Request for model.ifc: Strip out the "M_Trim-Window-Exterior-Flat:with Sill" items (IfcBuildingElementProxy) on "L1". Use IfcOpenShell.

First a look at what the model holds.

```python
import ifcopenshell
import ifcopenshell.util.element

model = ifcopenshell.open("model.ifc")
print(model.schema)
storey = next(s for s in model.by_type("IfcBuildingStorey") if s.Name == "L1")
proxies = [e for e in ifcopenshell.util.element.get_decomposition(storey) if e.is_a("IfcBuildingElementProxy")]
seen = {}
for e in proxies:
    element_type = ifcopenshell.util.element.get_type(e)
    name = element_type.Name if element_type not in (None, e) else None
    seen[name] = seen.get(name, 0) + 1
for name, count in sorted(seen.items(), key=str):
    print(count, "x", name)
```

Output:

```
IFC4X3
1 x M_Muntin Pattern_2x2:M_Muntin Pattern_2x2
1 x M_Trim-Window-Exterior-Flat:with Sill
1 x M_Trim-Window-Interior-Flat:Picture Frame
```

```python
import ifcopenshell
import ifcopenshell.api.root
import ifcopenshell.util.element

model = ifcopenshell.open("model.ifc")

storey = next(s for s in model.by_type("IfcBuildingStorey") if s.Name == "L1")
proxies = [e for e in ifcopenshell.util.element.get_decomposition(storey) if e.is_a("IfcBuildingElementProxy")]
targets = [e for e in proxies if (t := ifcopenshell.util.element.get_type(e)) not in (None, e) and t.Name == "M_Trim-Window-Exterior-Flat:with Sill"]

for e in targets:
    ifcopenshell.api.root.remove_product(model, product=e)
print(len(targets), "removed")

model.write("model-out.ifc")
```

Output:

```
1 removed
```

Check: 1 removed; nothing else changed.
